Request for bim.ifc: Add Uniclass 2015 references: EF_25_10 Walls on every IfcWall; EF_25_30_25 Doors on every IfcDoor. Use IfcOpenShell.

First a look at what the model holds.

```python
import ifcopenshell

model = ifcopenshell.open("bim.ifc")
print(model.schema)
print("classifications:", [c.Name for c in model.by_type("IfcClassification")])
for ifc_class in ("IfcDoor", "IfcRoof", "IfcStair", "IfcWall", "IfcWindow"):
    print(ifc_class, len(model.by_type(ifc_class)))
```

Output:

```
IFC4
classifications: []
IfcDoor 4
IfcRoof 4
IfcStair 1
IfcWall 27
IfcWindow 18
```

```python
import ifcopenshell
import ifcopenshell.api.classification

model = ifcopenshell.open("bim.ifc")

system = ifcopenshell.api.classification.add_classification(model, classification="Uniclass 2015")

codes = {
    "IfcWall": ("EF_25_10", "Walls"),
    "IfcDoor": ("EF_25_30_25", "Doors"),
}
for ifc_class, (code, name) in codes.items():
    products = model.by_type(ifc_class)
    ifcopenshell.api.classification.add_reference(
        model, products=products, classification=system, identification=code, name=name
    )
    print(code, len(products))

model.write("bim_updated.ifc")
```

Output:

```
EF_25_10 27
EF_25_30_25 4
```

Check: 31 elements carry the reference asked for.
